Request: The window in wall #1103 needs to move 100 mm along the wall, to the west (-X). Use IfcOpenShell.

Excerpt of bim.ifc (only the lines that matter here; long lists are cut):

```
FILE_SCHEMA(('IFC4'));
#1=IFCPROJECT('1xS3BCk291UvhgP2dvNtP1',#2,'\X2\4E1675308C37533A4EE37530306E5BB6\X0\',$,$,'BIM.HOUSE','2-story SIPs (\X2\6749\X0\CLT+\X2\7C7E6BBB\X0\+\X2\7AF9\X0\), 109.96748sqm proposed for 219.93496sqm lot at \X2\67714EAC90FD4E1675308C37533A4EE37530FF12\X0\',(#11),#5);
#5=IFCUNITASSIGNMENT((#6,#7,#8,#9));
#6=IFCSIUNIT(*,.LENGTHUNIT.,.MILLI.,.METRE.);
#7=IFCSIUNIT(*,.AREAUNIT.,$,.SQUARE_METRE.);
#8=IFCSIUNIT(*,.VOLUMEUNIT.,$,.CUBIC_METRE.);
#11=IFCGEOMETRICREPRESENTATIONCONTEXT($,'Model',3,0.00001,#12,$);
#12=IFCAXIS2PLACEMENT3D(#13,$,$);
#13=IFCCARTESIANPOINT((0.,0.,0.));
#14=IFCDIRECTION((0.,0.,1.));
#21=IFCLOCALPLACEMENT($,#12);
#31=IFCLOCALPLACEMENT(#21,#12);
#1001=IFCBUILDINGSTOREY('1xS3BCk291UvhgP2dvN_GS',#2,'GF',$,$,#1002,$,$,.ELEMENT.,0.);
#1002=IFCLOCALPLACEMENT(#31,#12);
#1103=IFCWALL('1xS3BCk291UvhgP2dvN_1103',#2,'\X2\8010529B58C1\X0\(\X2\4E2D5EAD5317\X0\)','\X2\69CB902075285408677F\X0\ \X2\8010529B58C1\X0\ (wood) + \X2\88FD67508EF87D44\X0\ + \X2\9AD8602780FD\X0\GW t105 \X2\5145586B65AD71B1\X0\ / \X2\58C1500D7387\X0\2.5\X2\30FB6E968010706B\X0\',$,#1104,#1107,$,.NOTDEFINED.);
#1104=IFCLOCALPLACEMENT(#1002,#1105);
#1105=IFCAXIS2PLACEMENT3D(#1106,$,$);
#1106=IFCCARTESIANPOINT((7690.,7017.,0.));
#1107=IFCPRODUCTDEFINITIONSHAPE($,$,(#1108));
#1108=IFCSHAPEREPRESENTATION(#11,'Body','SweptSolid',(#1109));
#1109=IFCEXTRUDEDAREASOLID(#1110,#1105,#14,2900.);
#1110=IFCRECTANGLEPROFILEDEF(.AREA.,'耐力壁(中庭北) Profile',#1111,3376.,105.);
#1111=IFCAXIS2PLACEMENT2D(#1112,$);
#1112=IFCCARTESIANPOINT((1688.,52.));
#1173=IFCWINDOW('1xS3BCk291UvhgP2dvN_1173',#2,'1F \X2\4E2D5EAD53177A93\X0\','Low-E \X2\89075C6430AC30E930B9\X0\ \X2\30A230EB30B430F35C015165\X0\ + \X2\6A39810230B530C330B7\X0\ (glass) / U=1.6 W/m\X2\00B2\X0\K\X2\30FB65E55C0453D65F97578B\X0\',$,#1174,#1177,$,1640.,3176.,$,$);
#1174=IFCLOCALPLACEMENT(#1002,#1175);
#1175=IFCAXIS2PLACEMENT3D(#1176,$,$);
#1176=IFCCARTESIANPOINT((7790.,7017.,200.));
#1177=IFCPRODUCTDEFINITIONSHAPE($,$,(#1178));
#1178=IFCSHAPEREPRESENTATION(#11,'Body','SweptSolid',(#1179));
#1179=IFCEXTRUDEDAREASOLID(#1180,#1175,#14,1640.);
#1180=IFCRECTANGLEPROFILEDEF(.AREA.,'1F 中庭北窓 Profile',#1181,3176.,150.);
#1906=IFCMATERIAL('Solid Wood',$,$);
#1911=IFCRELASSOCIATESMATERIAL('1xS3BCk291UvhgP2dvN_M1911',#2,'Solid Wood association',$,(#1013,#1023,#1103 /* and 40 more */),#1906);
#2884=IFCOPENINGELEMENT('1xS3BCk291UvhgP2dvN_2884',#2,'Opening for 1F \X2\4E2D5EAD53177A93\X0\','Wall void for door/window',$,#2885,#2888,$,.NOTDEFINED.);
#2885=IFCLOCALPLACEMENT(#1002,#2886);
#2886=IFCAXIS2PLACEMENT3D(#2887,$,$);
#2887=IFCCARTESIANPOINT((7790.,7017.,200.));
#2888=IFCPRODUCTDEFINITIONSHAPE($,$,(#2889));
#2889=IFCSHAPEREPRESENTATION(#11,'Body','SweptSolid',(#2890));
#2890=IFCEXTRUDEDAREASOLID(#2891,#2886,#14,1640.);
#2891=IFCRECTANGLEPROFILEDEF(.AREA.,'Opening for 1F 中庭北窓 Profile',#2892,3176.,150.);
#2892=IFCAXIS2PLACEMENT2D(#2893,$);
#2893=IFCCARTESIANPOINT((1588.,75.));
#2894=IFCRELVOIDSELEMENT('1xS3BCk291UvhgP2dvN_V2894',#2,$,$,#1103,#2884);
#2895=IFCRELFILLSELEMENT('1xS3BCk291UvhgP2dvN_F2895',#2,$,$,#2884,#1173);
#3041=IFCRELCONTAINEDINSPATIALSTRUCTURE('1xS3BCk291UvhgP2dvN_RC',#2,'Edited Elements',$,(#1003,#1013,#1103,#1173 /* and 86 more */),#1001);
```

```python
import ifcopenshell
import ifcopenshell.api.geometry
import ifcopenshell.util.placement
import ifcopenshell.util.unit

model = ifcopenshell.open("bim.ifc")
unit_scale = ifcopenshell.util.unit.calculate_unit_scale(model)

window = model.by_id(1173)
opening = window.FillsVoids[0].RelatingOpeningElement
wall = opening.VoidsElements[0].RelatingBuildingElement

wall_matrix = ifcopenshell.util.placement.get_local_placement(wall.ObjectPlacement)
shift = wall_matrix[:3, 0] * -0.1 / unit_scale
before = ifcopenshell.util.placement.get_local_placement(window.ObjectPlacement)[:3, 3].copy()

# The window is not placed relative to its opening, so move both.
for product in (opening, window):
    matrix = ifcopenshell.util.placement.get_local_placement(product.ObjectPlacement)
    matrix[:3, 3] += shift
    ifcopenshell.api.geometry.edit_object_placement(model, product=product, matrix=matrix, is_si=False)

after = ifcopenshell.util.placement.get_local_placement(window.ObjectPlacement)[:3, 3]
print("window moved by", (after - before).round(3) + 0.0)

model.write("bim_v2.ifc")
```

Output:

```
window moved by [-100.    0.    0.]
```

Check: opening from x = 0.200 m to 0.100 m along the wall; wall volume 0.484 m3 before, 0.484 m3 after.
